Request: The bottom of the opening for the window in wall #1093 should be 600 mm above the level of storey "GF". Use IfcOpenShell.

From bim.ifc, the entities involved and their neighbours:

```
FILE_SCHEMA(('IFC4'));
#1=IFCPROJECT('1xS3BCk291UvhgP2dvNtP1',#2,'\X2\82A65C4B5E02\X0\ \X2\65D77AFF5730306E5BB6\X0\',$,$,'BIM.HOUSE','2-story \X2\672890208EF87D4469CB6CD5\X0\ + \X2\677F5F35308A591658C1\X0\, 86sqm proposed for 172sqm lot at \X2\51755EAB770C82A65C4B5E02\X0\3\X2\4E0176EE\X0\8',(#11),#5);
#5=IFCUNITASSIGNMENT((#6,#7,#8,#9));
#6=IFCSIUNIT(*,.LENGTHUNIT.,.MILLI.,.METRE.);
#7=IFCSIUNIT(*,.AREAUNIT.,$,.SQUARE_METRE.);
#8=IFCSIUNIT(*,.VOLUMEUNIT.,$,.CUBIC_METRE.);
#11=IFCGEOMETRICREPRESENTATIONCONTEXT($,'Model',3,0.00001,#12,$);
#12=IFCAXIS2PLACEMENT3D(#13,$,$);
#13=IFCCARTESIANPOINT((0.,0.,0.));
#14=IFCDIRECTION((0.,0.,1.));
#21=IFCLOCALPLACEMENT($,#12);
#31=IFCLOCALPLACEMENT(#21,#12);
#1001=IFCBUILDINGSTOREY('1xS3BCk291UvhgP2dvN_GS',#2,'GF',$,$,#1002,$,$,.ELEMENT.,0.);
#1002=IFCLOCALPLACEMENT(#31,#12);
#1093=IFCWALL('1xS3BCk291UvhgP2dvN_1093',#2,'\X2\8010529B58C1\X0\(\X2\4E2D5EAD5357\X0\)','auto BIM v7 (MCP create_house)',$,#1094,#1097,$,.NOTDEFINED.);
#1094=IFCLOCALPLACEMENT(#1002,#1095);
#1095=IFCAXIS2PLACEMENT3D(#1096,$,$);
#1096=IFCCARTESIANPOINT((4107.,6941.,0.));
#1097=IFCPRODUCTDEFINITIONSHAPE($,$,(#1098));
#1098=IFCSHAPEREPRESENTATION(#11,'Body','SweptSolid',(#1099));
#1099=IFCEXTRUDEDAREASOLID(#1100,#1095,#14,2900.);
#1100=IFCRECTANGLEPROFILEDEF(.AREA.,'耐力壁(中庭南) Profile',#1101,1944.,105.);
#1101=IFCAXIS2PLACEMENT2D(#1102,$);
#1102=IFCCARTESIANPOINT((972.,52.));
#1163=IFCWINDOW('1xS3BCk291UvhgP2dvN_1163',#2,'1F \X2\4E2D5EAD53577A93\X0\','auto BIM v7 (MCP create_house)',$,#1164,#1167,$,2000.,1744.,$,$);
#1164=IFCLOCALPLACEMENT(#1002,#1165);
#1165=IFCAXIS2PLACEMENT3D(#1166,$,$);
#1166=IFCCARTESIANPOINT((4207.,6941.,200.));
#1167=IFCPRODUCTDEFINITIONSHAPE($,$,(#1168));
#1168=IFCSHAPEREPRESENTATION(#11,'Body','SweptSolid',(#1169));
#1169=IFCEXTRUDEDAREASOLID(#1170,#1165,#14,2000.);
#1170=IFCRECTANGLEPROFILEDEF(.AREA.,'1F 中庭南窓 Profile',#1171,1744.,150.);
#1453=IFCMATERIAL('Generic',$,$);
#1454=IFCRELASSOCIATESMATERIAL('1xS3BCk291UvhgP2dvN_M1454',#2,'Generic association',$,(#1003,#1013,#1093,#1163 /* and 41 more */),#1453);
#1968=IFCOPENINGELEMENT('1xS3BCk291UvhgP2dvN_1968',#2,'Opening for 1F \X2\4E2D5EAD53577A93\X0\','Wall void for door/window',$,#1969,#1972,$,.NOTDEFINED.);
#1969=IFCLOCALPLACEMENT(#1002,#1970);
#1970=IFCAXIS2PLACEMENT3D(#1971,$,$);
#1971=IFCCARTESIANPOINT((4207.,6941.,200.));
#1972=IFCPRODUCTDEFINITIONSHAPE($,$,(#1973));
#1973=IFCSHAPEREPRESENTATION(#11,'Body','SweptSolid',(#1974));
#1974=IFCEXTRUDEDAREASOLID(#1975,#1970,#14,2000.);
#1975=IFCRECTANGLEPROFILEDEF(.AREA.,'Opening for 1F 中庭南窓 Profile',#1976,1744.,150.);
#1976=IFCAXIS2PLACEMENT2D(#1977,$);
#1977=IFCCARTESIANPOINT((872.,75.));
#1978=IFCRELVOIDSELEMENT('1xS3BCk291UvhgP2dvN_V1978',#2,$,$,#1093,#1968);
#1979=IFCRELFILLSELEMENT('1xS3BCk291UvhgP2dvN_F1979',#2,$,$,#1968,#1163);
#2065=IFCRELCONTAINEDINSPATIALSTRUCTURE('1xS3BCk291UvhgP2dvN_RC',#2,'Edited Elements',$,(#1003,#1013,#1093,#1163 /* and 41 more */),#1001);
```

```python
import numpy as np
import ifcopenshell
import ifcopenshell.api.geometry
import ifcopenshell.geom
import ifcopenshell.util.element
import ifcopenshell.util.placement
import ifcopenshell.util.shape
import ifcopenshell.util.unit

model = ifcopenshell.open("bim.ifc")
unit_scale = ifcopenshell.util.unit.calculate_unit_scale(model)

window = model.by_guid("1xS3BCk291UvhgP2dvN_1163")
opening = window.FillsVoids[0].RelatingOpeningElement
storey = ifcopenshell.util.element.get_container(window, ifc_class="IfcBuildingStorey")
level = ifcopenshell.util.placement.get_local_placement(storey.ObjectPlacement)[2, 3]

# The opening's origin need not be at the sill, so measure its lowest point.
shape = ifcopenshell.geom.create_shape(ifcopenshell.geom.settings(), opening)
bottom = ifcopenshell.util.shape.get_shape_bottom_elevation(shape, shape.geometry) / unit_scale
dz = level + 0.6 / unit_scale - bottom

shift = np.array([0.0, 0.0, dz])
# The window is not placed relative to its opening, so move both.
for product in (opening, window):
    matrix = ifcopenshell.util.placement.get_local_placement(product.ObjectPlacement)
    matrix[:3, 3] += shift
    ifcopenshell.api.geometry.edit_object_placement(model, product=product, matrix=matrix, is_si=False)

print(f"moved by {dz * unit_scale:+.3f} m")

model.write("bim_edited.ifc")
```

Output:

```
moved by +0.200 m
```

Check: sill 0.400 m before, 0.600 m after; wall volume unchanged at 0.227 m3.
